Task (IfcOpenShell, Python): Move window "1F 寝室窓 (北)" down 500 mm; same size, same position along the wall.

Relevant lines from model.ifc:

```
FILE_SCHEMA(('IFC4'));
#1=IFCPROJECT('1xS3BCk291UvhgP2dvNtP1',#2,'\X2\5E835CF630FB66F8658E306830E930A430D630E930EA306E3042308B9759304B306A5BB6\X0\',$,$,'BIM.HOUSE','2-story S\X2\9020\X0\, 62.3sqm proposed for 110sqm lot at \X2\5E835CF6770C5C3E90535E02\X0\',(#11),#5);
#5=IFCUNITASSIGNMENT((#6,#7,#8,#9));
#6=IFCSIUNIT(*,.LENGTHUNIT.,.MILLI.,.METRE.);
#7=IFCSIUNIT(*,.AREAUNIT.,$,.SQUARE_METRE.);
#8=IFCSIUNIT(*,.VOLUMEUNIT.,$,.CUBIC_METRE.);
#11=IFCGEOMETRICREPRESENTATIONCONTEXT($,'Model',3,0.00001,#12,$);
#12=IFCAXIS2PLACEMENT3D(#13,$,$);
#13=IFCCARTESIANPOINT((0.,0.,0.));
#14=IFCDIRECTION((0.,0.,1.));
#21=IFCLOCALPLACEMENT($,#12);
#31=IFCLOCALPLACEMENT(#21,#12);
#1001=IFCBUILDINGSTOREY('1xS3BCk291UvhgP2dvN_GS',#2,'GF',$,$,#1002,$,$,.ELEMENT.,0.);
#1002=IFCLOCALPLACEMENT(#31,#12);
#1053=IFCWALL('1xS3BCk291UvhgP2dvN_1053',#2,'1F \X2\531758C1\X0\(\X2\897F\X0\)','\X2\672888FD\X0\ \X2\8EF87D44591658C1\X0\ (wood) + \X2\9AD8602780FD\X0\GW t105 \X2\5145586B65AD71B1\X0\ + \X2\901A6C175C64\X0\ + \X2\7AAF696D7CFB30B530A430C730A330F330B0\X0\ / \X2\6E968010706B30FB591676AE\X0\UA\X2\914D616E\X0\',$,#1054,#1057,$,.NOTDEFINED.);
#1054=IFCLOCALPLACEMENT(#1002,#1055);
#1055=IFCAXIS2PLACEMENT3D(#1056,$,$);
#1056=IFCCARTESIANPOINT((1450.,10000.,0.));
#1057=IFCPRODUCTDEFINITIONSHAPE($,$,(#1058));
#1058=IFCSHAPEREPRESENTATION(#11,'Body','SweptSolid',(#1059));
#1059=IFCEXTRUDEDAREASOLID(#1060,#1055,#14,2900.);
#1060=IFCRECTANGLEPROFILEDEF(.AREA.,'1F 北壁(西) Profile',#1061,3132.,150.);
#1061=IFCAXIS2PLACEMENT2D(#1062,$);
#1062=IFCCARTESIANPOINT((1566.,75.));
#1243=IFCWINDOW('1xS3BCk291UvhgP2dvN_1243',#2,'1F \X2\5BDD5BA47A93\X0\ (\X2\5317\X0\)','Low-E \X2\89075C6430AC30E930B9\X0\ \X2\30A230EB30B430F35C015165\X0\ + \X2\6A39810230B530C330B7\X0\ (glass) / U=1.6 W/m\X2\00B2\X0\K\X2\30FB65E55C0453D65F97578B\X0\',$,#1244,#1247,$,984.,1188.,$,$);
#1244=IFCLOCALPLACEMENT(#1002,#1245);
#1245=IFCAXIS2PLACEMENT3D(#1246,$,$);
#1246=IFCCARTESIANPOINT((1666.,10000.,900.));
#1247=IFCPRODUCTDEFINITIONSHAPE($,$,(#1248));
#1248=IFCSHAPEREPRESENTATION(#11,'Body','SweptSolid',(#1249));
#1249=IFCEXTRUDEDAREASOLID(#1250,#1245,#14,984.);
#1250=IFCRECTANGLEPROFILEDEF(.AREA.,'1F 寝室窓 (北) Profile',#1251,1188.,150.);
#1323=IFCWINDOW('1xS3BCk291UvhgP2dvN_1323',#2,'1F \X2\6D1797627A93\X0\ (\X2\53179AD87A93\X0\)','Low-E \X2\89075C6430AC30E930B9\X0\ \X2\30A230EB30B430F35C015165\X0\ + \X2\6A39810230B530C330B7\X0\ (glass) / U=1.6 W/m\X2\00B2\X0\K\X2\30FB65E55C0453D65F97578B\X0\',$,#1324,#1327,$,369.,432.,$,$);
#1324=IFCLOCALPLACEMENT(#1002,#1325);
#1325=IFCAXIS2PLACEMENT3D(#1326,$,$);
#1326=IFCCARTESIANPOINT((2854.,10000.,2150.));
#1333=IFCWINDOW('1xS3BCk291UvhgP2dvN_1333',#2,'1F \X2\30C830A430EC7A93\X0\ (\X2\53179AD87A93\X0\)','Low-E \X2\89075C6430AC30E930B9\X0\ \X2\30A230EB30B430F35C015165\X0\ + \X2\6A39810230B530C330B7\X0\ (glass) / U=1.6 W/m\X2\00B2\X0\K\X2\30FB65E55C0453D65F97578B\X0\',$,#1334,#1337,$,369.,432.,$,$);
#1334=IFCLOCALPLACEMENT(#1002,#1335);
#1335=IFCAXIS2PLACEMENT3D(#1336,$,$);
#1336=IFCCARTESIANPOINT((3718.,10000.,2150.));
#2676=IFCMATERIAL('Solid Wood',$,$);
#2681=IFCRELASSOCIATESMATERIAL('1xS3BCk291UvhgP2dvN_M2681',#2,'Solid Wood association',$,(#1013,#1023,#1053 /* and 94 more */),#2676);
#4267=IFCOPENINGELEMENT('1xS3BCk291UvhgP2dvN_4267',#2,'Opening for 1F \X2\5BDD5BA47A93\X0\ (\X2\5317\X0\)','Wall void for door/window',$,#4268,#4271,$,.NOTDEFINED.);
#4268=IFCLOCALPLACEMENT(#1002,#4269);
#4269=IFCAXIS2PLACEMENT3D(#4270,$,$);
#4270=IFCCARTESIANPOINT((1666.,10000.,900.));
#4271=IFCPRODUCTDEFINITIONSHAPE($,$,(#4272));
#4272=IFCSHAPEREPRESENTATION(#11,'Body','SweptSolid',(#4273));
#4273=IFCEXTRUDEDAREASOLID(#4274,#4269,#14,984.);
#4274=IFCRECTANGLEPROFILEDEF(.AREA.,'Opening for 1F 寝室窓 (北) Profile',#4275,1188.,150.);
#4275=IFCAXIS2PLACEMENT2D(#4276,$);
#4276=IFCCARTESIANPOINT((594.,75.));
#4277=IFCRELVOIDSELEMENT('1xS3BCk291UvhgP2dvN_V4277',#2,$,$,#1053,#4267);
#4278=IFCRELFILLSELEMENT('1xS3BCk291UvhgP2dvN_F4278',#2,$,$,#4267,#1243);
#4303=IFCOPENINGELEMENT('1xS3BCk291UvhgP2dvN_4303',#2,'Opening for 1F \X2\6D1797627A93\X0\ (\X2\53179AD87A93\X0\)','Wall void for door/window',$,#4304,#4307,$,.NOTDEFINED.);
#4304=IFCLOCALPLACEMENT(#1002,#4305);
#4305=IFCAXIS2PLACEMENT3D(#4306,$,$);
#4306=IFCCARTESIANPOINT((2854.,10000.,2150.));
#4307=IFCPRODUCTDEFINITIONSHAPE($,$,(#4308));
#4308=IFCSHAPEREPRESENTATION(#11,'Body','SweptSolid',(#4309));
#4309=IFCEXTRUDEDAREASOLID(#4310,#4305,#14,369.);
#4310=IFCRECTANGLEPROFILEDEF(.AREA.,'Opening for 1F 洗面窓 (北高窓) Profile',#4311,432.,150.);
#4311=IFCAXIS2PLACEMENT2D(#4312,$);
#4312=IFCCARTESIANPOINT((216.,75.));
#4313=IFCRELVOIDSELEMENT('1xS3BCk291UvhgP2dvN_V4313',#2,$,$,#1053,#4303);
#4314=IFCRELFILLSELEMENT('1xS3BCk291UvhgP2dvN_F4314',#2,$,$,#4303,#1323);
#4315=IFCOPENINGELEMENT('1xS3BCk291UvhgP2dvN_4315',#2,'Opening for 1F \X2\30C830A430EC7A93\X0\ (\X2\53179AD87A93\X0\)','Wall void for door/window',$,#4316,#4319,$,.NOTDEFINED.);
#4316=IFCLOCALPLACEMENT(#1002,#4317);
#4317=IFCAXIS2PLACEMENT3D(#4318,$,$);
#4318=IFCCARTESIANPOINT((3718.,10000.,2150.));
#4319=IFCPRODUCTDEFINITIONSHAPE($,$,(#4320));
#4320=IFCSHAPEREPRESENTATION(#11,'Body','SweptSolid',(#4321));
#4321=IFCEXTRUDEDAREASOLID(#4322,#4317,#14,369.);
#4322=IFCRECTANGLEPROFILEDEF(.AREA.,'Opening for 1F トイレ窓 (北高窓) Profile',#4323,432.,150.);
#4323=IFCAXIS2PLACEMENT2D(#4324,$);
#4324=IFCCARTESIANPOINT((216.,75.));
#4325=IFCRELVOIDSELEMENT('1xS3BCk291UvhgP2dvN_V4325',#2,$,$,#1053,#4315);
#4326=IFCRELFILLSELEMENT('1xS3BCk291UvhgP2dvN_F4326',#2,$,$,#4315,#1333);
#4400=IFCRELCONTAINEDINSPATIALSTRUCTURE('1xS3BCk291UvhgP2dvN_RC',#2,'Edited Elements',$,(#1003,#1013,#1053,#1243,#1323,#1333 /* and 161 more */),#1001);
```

```python
import numpy as np
import ifcopenshell
import ifcopenshell.api.geometry
import ifcopenshell.util.placement
import ifcopenshell.util.unit

model = ifcopenshell.open("model.ifc")
unit_scale = ifcopenshell.util.unit.calculate_unit_scale(model)

window = model.by_guid("1xS3BCk291UvhgP2dvN_1243")
opening = window.FillsVoids[0].RelatingOpeningElement
dz = -0.5 / unit_scale

shift = np.array([0.0, 0.0, dz])
# The window is not placed relative to its opening, so move both.
for product in (opening, window):
    matrix = ifcopenshell.util.placement.get_local_placement(product.ObjectPlacement)
    matrix[:3, 3] += shift
    ifcopenshell.api.geometry.edit_object_placement(model, product=product, matrix=matrix, is_si=False)

print(f"moved by {dz * unit_scale:+.3f} m")

model.write("model_v2.ifc")
```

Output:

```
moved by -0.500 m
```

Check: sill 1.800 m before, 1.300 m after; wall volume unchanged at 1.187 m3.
